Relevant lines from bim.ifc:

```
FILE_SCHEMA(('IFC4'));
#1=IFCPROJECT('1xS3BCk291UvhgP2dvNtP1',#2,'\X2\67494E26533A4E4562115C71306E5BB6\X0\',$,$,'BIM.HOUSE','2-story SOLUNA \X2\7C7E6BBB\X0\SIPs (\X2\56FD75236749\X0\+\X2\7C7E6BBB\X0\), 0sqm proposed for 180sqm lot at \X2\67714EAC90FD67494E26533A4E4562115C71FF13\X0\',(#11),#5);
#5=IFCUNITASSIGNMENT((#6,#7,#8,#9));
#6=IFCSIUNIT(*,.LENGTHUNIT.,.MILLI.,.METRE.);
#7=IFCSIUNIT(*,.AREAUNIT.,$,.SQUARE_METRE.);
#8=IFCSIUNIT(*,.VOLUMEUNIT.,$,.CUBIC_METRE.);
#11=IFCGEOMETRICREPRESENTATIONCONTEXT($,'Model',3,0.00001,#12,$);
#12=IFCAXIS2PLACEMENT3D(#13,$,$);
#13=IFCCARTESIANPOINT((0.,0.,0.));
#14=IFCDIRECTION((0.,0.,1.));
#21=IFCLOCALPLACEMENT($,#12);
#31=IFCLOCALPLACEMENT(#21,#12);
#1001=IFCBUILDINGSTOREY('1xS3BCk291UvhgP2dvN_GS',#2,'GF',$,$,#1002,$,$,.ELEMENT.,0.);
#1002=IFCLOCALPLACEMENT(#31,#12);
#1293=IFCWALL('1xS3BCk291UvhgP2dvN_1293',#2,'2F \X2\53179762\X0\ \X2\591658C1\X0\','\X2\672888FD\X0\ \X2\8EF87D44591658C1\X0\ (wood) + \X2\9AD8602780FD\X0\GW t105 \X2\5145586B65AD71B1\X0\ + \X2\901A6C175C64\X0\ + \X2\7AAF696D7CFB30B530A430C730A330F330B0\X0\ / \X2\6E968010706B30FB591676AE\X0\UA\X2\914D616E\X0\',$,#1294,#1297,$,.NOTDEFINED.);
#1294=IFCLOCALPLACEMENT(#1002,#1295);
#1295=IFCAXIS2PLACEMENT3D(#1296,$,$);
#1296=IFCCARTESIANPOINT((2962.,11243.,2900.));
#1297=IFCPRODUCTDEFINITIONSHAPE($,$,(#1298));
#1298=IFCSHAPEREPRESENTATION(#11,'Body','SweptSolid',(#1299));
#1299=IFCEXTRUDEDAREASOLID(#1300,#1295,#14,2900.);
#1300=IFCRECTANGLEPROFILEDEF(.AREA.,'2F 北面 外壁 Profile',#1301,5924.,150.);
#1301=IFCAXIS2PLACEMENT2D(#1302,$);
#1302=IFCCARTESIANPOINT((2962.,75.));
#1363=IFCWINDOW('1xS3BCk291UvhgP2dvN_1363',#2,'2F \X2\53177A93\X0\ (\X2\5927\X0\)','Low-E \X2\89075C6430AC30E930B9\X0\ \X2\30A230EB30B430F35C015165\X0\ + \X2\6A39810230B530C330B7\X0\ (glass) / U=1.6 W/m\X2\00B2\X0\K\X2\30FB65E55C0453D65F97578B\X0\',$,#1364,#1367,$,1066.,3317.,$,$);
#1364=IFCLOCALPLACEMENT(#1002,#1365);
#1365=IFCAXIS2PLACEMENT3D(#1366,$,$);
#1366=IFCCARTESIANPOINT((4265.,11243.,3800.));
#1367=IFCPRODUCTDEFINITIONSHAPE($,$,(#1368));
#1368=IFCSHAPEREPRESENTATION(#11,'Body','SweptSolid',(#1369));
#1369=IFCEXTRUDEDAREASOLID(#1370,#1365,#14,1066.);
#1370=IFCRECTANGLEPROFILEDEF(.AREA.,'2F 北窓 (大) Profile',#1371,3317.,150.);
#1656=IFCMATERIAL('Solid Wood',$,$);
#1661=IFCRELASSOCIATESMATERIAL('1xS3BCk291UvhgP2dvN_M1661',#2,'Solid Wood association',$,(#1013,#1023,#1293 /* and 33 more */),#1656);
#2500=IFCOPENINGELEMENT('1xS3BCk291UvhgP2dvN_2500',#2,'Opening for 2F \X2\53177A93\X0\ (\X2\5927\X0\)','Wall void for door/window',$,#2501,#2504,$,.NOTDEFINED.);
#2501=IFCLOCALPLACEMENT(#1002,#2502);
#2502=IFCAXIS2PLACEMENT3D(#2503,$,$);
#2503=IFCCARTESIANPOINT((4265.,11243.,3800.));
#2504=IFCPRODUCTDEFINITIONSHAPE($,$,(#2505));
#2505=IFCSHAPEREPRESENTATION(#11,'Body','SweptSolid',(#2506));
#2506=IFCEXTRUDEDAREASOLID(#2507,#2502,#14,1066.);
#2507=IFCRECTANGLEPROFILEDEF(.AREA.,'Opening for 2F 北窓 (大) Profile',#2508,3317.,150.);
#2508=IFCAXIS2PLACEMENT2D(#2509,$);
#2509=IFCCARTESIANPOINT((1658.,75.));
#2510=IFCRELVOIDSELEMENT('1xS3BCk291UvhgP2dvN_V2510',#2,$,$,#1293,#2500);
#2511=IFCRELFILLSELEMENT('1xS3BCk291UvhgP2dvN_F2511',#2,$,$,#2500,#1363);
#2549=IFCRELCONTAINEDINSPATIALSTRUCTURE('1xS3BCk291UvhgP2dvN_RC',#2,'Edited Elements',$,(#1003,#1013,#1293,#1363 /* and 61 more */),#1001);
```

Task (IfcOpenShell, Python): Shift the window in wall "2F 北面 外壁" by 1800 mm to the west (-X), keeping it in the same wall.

```python
import ifcopenshell
import ifcopenshell.api.geometry
import ifcopenshell.util.placement

model = ifcopenshell.open("bim.ifc")

window = model.by_guid("1xS3BCk291UvhgP2dvN_1363")
opening = window.FillsVoids[0].RelatingOpeningElement
wall = opening.VoidsElements[0].RelatingBuildingElement

wall_matrix = ifcopenshell.util.placement.get_local_placement(wall.ObjectPlacement)
shift = wall_matrix[:3, 0] * -1800.0
before = ifcopenshell.util.placement.get_local_placement(window.ObjectPlacement)[:3, 3].copy()

# The window is not placed relative to its opening, so move both.
for product in (opening, window):
    matrix = ifcopenshell.util.placement.get_local_placement(product.ObjectPlacement)
    matrix[:3, 3] += shift
    ifcopenshell.api.geometry.edit_object_placement(model, product=product, matrix=matrix, is_si=False)

after = ifcopenshell.util.placement.get_local_placement(window.ObjectPlacement)[:3, 3]
print("window moved by", (after - before).round(3) + 0.0)

model.write("bim_rev.ifc")
```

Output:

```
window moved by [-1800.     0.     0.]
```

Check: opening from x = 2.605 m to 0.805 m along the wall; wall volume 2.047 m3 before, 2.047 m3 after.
